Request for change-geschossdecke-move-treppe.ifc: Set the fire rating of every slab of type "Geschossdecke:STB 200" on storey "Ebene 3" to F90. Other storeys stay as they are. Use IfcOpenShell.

First a look at what the model holds.

```python
import ifcopenshell
import ifcopenshell.util.element

model = ifcopenshell.open("change-geschossdecke-move-treppe.ifc")
print(model.schema)
storey = next(s for s in model.by_type("IfcBuildingStorey") if s.Name == "Ebene 3")
slabs = [e for e in ifcopenshell.util.element.get_decomposition(storey) if e.is_a("IfcSlab")]
seen = {}
for e in slabs:
    element_type = ifcopenshell.util.element.get_type(e)
    key = (element_type.Name if element_type != e and element_type else None, ifcopenshell.util.element.get_pset(e, "Pset_SlabCommon", "FireRating"))
    seen[key] = seen.get(key, 0) + 1
for (name, value), count in sorted(seen.items(), key=str):
    print(count, "x", name, "|", value)
```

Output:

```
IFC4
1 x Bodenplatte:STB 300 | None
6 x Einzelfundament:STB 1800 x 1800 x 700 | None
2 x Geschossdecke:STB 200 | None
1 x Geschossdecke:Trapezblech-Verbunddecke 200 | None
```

```python
import ifcopenshell
import ifcopenshell.api.pset
import ifcopenshell.util.element

model = ifcopenshell.open("change-geschossdecke-move-treppe.ifc")

storey = next(s for s in model.by_type("IfcBuildingStorey") if s.Name == "Ebene 3")
slabs = [e for e in ifcopenshell.util.element.get_decomposition(storey) if e.is_a("IfcSlab")]

count = 0
for e in slabs:
    element_type = ifcopenshell.util.element.get_type(e)
    if element_type in (None, e) or element_type.Name != "Geschossdecke:STB 200":
        continue
    # add_pset returns the element's existing set when there is one.
    pset = ifcopenshell.api.pset.add_pset(model, product=e, name="Pset_SlabCommon")
    ifcopenshell.api.pset.edit_pset(model, pset=pset, properties={"FireRating": "F90"})
    count += 1

print(count, "slabs updated")

model.write("change-geschossdecke-move-treppe_updated.ifc")
```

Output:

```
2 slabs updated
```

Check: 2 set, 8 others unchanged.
